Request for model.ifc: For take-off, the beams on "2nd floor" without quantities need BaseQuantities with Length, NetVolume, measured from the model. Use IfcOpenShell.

First a look at what the model holds.

```python
import ifcopenshell
import ifcopenshell.util.element
import ifcopenshell.util.unit

model = ifcopenshell.open("model.ifc")
print(model.schema)
for unit_type in ("LENGTHUNIT", "AREAUNIT", "VOLUMEUNIT"):
    print(unit_type, ifcopenshell.util.unit.calculate_unit_scale(model, unit_type))
storey = next(s for s in model.by_type("IfcBuildingStorey") if s.Name == "2nd floor")
beams = [e for e in ifcopenshell.util.element.get_decomposition(storey) if e.is_a("IfcBeam")]
for e in sorted(beams, key=lambda e: e.id()):
    print(e.id(), e.is_a(), e.Name, list(ifcopenshell.util.element.get_psets(e, qtos_only=True)), sep=" | ")
```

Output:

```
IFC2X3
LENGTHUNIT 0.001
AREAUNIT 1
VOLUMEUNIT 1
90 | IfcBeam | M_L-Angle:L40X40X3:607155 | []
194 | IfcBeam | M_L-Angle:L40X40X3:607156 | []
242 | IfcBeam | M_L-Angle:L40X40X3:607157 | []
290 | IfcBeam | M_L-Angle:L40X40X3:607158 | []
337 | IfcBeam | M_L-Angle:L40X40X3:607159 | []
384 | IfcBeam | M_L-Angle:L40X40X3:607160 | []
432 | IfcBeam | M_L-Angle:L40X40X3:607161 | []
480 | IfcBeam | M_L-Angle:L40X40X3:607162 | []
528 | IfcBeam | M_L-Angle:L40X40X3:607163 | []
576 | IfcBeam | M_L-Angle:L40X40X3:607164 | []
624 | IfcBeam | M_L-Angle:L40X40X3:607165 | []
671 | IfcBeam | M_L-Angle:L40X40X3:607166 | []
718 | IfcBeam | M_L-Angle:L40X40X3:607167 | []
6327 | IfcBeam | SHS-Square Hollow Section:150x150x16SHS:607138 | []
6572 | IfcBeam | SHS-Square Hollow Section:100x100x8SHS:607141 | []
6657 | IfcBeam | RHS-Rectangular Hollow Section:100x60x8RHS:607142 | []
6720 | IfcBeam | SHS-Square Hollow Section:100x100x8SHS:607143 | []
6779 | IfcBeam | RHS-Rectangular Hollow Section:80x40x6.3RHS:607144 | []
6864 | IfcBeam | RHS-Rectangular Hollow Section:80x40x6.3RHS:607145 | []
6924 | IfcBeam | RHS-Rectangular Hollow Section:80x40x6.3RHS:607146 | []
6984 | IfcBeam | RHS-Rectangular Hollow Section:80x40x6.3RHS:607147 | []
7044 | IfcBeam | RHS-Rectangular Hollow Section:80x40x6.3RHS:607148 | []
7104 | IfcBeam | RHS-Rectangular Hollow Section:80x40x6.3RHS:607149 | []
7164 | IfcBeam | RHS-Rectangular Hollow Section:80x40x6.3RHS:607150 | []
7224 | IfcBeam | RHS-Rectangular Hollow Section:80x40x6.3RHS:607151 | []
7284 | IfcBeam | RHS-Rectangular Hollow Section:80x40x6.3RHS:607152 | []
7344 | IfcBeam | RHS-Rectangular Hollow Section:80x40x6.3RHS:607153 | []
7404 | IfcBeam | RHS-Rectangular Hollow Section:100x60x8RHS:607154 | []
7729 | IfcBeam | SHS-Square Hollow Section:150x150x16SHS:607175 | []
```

```python
import ifcopenshell
import ifcopenshell.api.pset
import ifcopenshell.geom
import ifcopenshell.util.element
import ifcopenshell.util.shape
import ifcopenshell.util.unit

model = ifcopenshell.open("model.ifc")
unit_scale = ifcopenshell.util.unit.calculate_unit_scale(model)
volume_scale = ifcopenshell.util.unit.calculate_unit_scale(model, "VOLUMEUNIT")
settings = ifcopenshell.geom.settings()

storey = next(s for s in model.by_type("IfcBuildingStorey") if s.Name == "2nd floor")
beams = [e for e in ifcopenshell.util.element.get_decomposition(storey) if e.is_a("IfcBeam")]

for e in sorted(beams, key=lambda e: e.id()):
    if ifcopenshell.util.element.get_psets(e, qtos_only=True, should_inherit=False):
        continue
    # Geometry comes back in metres, in the element's own axes.
    shape = ifcopenshell.geom.create_shape(settings, e)
    values = {
        "Length": ifcopenshell.util.shape.get_max_xyz(shape.geometry) / unit_scale,
        "NetVolume": ifcopenshell.util.shape.get_volume(shape.geometry) / volume_scale,
    }
    qto = ifcopenshell.api.pset.add_qto(model, product=e, name="BaseQuantities")
    ifcopenshell.api.pset.edit_qto(model, qto=qto, properties=values)
    print(e.id(), {k: round(v, 3) for k, v in values.items()})

model.write("model_edited.ifc")
```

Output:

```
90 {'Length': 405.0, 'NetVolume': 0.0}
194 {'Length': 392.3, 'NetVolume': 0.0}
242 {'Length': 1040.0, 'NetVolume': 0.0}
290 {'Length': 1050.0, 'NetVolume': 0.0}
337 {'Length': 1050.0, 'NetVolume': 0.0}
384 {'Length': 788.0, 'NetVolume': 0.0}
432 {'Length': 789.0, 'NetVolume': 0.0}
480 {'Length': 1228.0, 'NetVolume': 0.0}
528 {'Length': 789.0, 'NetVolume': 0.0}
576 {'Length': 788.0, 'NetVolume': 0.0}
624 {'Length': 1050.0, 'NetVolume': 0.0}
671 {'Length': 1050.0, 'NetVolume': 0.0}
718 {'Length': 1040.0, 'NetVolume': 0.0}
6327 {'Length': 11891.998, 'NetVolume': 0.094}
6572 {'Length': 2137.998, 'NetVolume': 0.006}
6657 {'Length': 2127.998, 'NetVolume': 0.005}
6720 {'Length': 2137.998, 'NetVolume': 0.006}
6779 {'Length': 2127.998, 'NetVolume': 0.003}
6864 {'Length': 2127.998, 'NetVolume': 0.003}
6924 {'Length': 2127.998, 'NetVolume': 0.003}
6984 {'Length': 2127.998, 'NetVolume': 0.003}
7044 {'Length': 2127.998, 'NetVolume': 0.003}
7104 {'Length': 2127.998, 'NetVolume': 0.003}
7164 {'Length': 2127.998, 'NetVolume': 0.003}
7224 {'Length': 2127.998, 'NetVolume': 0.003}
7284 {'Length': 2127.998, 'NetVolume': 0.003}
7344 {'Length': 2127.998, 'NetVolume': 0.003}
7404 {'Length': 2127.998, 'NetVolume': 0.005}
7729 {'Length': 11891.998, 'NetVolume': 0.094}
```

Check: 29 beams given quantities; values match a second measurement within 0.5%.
